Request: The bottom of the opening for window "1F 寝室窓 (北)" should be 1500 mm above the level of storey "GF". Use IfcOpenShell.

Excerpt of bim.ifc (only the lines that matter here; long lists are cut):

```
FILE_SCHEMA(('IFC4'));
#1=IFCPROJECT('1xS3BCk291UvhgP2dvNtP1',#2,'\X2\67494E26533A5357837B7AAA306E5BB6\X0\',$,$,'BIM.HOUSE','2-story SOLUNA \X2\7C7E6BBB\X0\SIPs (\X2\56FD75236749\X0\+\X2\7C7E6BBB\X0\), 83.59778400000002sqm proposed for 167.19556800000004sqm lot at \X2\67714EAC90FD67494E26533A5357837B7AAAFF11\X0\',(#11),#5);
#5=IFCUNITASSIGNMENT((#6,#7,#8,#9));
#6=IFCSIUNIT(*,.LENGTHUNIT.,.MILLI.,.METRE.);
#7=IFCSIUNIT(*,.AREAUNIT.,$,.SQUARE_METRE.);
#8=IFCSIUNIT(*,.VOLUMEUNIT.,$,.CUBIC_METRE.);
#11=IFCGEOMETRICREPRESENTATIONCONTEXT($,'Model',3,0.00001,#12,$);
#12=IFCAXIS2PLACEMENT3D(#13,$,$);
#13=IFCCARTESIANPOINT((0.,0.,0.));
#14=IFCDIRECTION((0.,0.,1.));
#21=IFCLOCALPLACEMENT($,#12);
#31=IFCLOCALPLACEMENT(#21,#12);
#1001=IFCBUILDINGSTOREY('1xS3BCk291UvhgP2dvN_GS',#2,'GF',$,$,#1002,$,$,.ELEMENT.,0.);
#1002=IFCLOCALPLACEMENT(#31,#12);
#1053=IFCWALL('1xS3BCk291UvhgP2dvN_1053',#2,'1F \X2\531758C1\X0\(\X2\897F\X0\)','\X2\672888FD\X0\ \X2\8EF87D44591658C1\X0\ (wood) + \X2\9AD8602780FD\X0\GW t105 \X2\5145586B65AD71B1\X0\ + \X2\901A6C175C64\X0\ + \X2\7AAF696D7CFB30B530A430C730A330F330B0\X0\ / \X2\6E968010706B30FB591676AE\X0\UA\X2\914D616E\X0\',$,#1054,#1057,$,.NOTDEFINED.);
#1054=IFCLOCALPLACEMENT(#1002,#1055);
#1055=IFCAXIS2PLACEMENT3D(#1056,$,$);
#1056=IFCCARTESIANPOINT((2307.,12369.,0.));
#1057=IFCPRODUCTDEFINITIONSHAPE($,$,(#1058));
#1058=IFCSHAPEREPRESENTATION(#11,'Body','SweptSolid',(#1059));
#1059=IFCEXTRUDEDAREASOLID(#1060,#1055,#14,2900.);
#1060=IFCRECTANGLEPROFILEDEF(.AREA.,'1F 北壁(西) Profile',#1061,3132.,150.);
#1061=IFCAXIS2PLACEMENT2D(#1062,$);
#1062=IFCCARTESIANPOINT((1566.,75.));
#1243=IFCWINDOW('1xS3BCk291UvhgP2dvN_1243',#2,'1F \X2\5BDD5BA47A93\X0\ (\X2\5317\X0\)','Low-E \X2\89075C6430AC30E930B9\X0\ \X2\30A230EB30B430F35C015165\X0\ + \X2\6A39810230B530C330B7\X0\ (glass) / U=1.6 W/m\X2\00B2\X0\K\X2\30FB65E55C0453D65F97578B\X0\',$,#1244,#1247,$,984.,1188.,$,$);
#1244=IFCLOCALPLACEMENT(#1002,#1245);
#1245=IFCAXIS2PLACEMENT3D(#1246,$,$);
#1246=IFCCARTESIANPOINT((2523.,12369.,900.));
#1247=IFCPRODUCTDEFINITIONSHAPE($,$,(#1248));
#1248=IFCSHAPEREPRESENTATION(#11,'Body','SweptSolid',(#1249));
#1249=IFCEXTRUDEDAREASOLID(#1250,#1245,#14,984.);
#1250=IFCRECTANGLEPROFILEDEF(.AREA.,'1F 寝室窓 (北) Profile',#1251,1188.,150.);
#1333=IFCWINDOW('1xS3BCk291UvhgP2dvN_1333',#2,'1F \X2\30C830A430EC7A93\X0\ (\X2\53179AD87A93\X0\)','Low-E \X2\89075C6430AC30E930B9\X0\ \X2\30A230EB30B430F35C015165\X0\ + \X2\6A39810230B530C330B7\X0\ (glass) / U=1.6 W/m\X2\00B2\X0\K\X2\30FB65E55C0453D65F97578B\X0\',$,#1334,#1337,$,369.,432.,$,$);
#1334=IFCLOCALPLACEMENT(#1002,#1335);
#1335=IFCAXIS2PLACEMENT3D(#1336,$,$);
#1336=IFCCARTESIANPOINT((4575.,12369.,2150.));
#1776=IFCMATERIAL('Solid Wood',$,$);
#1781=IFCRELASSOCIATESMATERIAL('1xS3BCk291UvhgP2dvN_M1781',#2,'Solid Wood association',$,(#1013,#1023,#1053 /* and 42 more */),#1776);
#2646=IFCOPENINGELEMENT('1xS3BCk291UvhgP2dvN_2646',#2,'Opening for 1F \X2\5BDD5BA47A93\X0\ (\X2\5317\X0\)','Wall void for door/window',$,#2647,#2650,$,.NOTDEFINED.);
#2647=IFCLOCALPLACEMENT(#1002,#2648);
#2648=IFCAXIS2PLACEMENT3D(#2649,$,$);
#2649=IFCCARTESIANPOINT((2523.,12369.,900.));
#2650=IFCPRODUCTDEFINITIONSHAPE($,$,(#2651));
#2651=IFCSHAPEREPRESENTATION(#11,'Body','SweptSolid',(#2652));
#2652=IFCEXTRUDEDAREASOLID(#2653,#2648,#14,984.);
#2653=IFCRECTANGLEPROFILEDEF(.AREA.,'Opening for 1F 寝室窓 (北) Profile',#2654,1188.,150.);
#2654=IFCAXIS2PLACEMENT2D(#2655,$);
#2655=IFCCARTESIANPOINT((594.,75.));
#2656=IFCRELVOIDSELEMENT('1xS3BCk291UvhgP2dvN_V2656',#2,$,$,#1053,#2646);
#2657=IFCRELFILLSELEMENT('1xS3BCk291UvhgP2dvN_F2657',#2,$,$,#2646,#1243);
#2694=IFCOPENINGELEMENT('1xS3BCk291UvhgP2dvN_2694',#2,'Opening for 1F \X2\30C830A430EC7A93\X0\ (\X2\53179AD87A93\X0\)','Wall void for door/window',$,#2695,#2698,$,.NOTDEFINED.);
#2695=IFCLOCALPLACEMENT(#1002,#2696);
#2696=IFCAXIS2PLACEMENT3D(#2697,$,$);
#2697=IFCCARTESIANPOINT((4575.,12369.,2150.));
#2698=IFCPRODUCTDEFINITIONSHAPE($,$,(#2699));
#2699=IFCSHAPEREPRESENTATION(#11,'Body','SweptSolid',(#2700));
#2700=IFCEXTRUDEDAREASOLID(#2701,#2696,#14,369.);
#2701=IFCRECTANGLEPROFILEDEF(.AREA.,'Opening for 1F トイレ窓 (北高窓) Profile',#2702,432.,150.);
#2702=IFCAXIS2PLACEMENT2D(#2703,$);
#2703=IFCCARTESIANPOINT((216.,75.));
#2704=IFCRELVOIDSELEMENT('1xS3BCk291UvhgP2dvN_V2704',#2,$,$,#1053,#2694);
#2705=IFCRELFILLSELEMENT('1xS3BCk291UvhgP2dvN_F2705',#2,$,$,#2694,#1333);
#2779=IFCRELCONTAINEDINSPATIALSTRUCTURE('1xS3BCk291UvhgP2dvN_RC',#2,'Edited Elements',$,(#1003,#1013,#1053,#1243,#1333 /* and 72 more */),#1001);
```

```python
import numpy as np
import ifcopenshell
import ifcopenshell.api.geometry
import ifcopenshell.geom
import ifcopenshell.util.element
import ifcopenshell.util.placement
import ifcopenshell.util.shape
import ifcopenshell.util.unit

model = ifcopenshell.open("bim.ifc")
unit_scale = ifcopenshell.util.unit.calculate_unit_scale(model)

window = model.by_id(1243)
opening = window.FillsVoids[0].RelatingOpeningElement
storey = ifcopenshell.util.element.get_container(window, ifc_class="IfcBuildingStorey")
level = ifcopenshell.util.placement.get_local_placement(storey.ObjectPlacement)[2, 3]

# The opening's origin need not be at the sill, so measure its lowest point.
shape = ifcopenshell.geom.create_shape(ifcopenshell.geom.settings(), opening)
bottom = ifcopenshell.util.shape.get_shape_bottom_elevation(shape, shape.geometry) / unit_scale
dz = level + 1500.0 - bottom

shift = np.array([0.0, 0.0, dz])
# The window is not placed relative to its opening, so move both.
for product in (opening, window):
    matrix = ifcopenshell.util.placement.get_local_placement(product.ObjectPlacement)
    matrix[:3, 3] += shift
    ifcopenshell.api.geometry.edit_object_placement(model, product=product, matrix=matrix, is_si=False)

print(f"moved by {dz * unit_scale:+.3f} m")

model.write("bim_updated.ifc")
```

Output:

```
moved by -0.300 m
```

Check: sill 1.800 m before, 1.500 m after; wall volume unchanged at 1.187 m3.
